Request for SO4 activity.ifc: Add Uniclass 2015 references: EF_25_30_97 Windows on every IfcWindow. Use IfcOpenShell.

First a look at what the model holds.

```python
import ifcopenshell

model = ifcopenshell.open("SO4 activity.ifc")
print(model.schema)
print("classifications:", [c.Name for c in model.by_type("IfcClassification")])
for ifc_class in ("IfcDoor", "IfcRoof", "IfcStair", "IfcWall", "IfcWindow"):
    print(ifc_class, len(model.by_type(ifc_class)))
```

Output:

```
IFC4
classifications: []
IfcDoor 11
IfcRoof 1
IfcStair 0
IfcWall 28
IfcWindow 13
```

```python
import ifcopenshell
import ifcopenshell.api.classification

model = ifcopenshell.open("SO4 activity.ifc")

system = ifcopenshell.api.classification.add_classification(model, classification="Uniclass 2015")

codes = {
    "IfcWindow": ("EF_25_30_97", "Windows"),
}
for ifc_class, (code, name) in codes.items():
    products = model.by_type(ifc_class)
    ifcopenshell.api.classification.add_reference(
        model, products=products, classification=system, identification=code, name=name
    )
    print(code, len(products))

model.write("SO4 activity_edited.ifc")
```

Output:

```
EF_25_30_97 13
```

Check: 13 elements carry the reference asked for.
